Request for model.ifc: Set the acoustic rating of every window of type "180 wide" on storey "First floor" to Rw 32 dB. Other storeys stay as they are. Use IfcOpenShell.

First a look at what the model holds.

```python
import ifcopenshell
import ifcopenshell.util.element

model = ifcopenshell.open("model.ifc")
print(model.schema)
storey = next(s for s in model.by_type("IfcBuildingStorey") if s.Name == "First floor")
windows = [e for e in ifcopenshell.util.element.get_decomposition(storey) if e.is_a("IfcWindow")]
seen = {}
for e in windows:
    element_type = ifcopenshell.util.element.get_type(e)
    key = (element_type.Name if element_type != e and element_type else None, ifcopenshell.util.element.get_pset(e, "Pset_WindowCommon", "AcousticRating"))
    seen[key] = seen.get(key, 0) + 1
for (name, value), count in sorted(seen.items(), key=str):
    print(count, "x", name, "|", value)
```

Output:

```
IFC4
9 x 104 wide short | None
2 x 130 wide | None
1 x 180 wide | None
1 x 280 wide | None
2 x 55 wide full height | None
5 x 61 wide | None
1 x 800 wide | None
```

```python
import ifcopenshell
import ifcopenshell.api.pset
import ifcopenshell.util.element

model = ifcopenshell.open("model.ifc")

storey = next(s for s in model.by_type("IfcBuildingStorey") if s.Name == "First floor")
windows = [e for e in ifcopenshell.util.element.get_decomposition(storey) if e.is_a("IfcWindow")]

count = 0
for e in windows:
    element_type = ifcopenshell.util.element.get_type(e)
    if element_type in (None, e) or element_type.Name != "180 wide":
        continue
    # add_pset returns the element's existing set when there is one.
    pset = ifcopenshell.api.pset.add_pset(model, product=e, name="Pset_WindowCommon")
    ifcopenshell.api.pset.edit_pset(model, pset=pset, properties={"AcousticRating": "Rw 32 dB"})
    count += 1

print(count, "windows updated")

model.write("model_edited.ifc")
```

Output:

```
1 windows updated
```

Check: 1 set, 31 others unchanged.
